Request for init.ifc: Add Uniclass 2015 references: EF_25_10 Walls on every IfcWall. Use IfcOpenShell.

First a look at what the model holds.

```python
import ifcopenshell

model = ifcopenshell.open("init.ifc")
print(model.schema)
print("classifications:", [c.Name for c in model.by_type("IfcClassification")])
for ifc_class in ("IfcDoor", "IfcRoof", "IfcStair", "IfcWall", "IfcWindow"):
    print(ifc_class, len(model.by_type(ifc_class)))
```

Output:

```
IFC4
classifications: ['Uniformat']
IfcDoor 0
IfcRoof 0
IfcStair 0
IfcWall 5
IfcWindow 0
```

```python
import ifcopenshell
import ifcopenshell.api.classification

model = ifcopenshell.open("init.ifc")

system = ifcopenshell.api.classification.add_classification(model, classification="Uniclass 2015")

codes = {
    "IfcWall": ("EF_25_10", "Walls"),
}
for ifc_class, (code, name) in codes.items():
    products = model.by_type(ifc_class)
    ifcopenshell.api.classification.add_reference(
        model, products=products, classification=system, identification=code, name=name
    )
    print(code, len(products))

model.write("init_v2.ifc")
```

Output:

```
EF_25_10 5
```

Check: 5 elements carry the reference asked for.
